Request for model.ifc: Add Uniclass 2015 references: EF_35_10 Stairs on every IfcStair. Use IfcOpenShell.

First a look at what the model holds.

```python
import ifcopenshell

model = ifcopenshell.open("model.ifc")
print(model.schema)
print("classifications:", [c.Name for c in model.by_type("IfcClassification")])
for ifc_class in ("IfcDoor", "IfcRoof", "IfcStair", "IfcWall", "IfcWindow"):
    print(ifc_class, len(model.by_type(ifc_class)))
```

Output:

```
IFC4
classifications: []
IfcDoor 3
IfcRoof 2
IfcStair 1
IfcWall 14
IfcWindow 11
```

```python
import ifcopenshell
import ifcopenshell.api.classification

model = ifcopenshell.open("model.ifc")

system = ifcopenshell.api.classification.add_classification(model, classification="Uniclass 2015")

codes = {
    "IfcStair": ("EF_35_10", "Stairs"),
}
for ifc_class, (code, name) in codes.items():
    products = model.by_type(ifc_class)
    ifcopenshell.api.classification.add_reference(
        model, products=products, classification=system, identification=code, name=name
    )
    print(code, len(products))

model.write("model_rev.ifc")
```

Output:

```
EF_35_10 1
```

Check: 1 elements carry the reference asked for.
